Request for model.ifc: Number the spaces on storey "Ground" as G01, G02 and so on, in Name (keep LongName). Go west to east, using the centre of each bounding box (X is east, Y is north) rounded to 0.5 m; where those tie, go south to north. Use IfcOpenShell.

First a look at what the model holds.

```python
import ifcopenshell
import ifcopenshell.util.element
import ifcopenshell.util.placement

model = ifcopenshell.open("model.ifc")
print(model.schema)
storey = next(s for s in model.by_type("IfcBuildingStorey") if s.Name == "Ground")
spaces = [e for e in ifcopenshell.util.element.get_decomposition(storey) if e.is_a("IfcSpace")]
for e in sorted(spaces, key=lambda e: e.id()):
    origin = ifcopenshell.util.placement.get_local_placement(e.ObjectPlacement)[:3, 3]
    print(e.id(), e.Name, e.LongName, origin.round(2) + 0.0, sep=" | ")
```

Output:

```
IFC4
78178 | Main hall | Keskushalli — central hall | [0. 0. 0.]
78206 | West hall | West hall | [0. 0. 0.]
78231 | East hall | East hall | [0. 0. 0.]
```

```python
import ifcopenshell
import ifcopenshell.geom
import ifcopenshell.util.element
import ifcopenshell.util.shape

model = ifcopenshell.open("model.ifc")
settings = ifcopenshell.geom.settings()
settings.set("use-world-coords", True)


def centre(element):
    shape = ifcopenshell.geom.create_shape(settings, element)
    return ifcopenshell.util.shape.get_bbox_centroid(shape.geometry)


storey = next(s for s in model.by_type("IfcBuildingStorey") if s.Name == "Ground")
spaces = [e for e in ifcopenshell.util.element.get_decomposition(storey) if e.is_a("IfcSpace")]

# Insertion points can sit at a corner or the storey origin, so sort by the geometry (in metres).
centres = {e: centre(e) for e in spaces}
spaces.sort(key=lambda e: (round(centres[e][0] / 0.5), centres[e][1]))

for i, e in enumerate(spaces, start=1):
    number = f"G{i:02d}"
    e.Name = number
    print(e.id(), number)

model.write("model-out.ifc")
```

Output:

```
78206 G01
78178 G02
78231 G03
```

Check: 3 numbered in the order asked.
